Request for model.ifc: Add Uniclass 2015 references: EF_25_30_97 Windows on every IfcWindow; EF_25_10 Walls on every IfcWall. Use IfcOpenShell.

First a look at what the model holds.

```python
import ifcopenshell

model = ifcopenshell.open("model.ifc")
print(model.schema)
print("classifications:", [c.Name for c in model.by_type("IfcClassification")])
for ifc_class in ("IfcDoor", "IfcRoof", "IfcStair", "IfcWall", "IfcWindow"):
    print(ifc_class, len(model.by_type(ifc_class)))
```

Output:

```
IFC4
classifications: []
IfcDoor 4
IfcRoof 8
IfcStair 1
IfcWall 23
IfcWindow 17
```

```python
import ifcopenshell
import ifcopenshell.api.classification

model = ifcopenshell.open("model.ifc")

system = ifcopenshell.api.classification.add_classification(model, classification="Uniclass 2015")

codes = {
    "IfcWindow": ("EF_25_30_97", "Windows"),
    "IfcWall": ("EF_25_10", "Walls"),
}
for ifc_class, (code, name) in codes.items():
    products = model.by_type(ifc_class)
    ifcopenshell.api.classification.add_reference(
        model, products=products, classification=system, identification=code, name=name
    )
    print(code, len(products))

model.write("model_v2.ifc")
```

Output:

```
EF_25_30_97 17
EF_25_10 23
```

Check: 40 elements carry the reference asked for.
